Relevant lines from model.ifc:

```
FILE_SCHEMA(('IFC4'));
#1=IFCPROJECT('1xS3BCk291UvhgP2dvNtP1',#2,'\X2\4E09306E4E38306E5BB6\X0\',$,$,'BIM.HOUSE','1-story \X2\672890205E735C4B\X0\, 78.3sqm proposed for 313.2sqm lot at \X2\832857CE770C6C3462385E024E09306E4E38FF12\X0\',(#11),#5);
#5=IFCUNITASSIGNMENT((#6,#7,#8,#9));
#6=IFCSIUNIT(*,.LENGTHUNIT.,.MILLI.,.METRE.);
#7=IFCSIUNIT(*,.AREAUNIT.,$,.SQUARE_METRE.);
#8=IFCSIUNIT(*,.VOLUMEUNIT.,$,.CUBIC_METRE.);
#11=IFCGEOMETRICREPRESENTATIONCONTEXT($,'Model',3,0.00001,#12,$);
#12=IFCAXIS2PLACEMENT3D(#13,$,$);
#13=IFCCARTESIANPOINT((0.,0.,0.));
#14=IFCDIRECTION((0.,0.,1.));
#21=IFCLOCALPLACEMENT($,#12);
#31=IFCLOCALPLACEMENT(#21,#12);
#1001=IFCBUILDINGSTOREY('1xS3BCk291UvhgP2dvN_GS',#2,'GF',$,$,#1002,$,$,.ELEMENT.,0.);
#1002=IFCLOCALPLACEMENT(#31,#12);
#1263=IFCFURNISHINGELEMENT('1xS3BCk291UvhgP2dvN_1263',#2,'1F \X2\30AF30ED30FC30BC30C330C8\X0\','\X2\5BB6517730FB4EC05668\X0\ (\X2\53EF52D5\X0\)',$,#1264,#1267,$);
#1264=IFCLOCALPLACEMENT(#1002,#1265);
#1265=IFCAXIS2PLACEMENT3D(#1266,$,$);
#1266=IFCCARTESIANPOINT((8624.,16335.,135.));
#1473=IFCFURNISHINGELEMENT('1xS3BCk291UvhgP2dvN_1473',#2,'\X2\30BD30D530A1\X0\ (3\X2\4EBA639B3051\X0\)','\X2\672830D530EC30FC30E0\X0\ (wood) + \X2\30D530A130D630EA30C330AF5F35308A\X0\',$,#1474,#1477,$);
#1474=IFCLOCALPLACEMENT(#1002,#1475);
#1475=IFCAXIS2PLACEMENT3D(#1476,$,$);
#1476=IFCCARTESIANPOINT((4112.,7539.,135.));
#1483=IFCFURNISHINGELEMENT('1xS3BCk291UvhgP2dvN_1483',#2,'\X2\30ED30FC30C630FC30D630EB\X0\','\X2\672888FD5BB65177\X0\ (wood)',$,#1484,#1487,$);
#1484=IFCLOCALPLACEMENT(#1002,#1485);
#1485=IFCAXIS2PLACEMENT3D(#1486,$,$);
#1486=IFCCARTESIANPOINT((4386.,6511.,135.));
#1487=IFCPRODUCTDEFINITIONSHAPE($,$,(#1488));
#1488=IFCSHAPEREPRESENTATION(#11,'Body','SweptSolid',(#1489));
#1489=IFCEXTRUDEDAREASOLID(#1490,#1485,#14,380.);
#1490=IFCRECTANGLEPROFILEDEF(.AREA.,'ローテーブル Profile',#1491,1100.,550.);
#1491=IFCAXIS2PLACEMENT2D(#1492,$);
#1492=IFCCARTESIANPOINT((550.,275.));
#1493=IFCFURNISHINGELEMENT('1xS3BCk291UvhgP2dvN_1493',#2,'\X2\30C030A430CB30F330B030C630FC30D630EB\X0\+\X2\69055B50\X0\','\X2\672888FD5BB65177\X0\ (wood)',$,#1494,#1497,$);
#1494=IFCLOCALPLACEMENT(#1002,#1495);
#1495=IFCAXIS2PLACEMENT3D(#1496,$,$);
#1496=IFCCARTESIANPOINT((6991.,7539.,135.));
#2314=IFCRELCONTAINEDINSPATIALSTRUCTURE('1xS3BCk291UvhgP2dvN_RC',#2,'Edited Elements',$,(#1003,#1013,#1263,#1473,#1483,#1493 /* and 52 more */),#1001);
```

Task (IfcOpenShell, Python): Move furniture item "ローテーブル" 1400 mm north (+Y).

```python
import ifcopenshell
import ifcopenshell.api.geometry
import ifcopenshell.util.placement
import ifcopenshell.util.unit

model = ifcopenshell.open("model.ifc")
unit_scale = ifcopenshell.util.unit.calculate_unit_scale(model)

item = model.by_guid("1xS3BCk291UvhgP2dvN_1483")
matrix = ifcopenshell.util.placement.get_local_placement(item.ObjectPlacement)
matrix[1, 3] += 1.4 / unit_scale
ifcopenshell.api.geometry.edit_object_placement(model, product=item, matrix=matrix, is_si=False)

print(ifcopenshell.util.placement.get_local_placement(item.ObjectPlacement).round(3) + 0.0)

model.write("model_v2.ifc")
```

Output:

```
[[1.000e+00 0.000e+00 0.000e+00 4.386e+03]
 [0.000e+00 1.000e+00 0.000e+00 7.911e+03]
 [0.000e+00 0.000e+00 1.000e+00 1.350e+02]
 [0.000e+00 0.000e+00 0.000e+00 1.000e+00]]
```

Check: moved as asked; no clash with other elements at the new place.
